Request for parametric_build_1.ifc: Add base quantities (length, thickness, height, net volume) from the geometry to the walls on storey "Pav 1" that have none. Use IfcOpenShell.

First a look at what the model holds.

```python
import ifcopenshell
import ifcopenshell.util.element
import ifcopenshell.util.unit

model = ifcopenshell.open("parametric_build_1.ifc")
print(model.schema)
for unit_type in ("LENGTHUNIT", "AREAUNIT", "VOLUMEUNIT"):
    print(unit_type, ifcopenshell.util.unit.calculate_unit_scale(model, unit_type))
storey = next(s for s in model.by_type("IfcBuildingStorey") if s.Name == "Pav 1")
walls = [e for e in ifcopenshell.util.element.get_decomposition(storey) if e.is_a("IfcWall")]
for e in sorted(walls, key=lambda e: e.id()):
    print(e.id(), e.is_a(), e.Name, list(ifcopenshell.util.element.get_psets(e, qtos_only=True)), sep=" | ")
```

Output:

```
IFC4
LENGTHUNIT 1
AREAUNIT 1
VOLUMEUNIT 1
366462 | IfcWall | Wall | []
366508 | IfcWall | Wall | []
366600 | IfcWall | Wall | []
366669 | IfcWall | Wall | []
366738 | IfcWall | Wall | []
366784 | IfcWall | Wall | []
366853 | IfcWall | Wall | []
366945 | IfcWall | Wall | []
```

```python
import ifcopenshell
import ifcopenshell.api.pset
import ifcopenshell.geom
import ifcopenshell.util.element
import ifcopenshell.util.shape
import ifcopenshell.util.unit

model = ifcopenshell.open("parametric_build_1.ifc")
unit_scale = ifcopenshell.util.unit.calculate_unit_scale(model)
volume_scale = ifcopenshell.util.unit.calculate_unit_scale(model, "VOLUMEUNIT")
settings = ifcopenshell.geom.settings()

storey = next(s for s in model.by_type("IfcBuildingStorey") if s.Name == "Pav 1")
walls = [e for e in ifcopenshell.util.element.get_decomposition(storey) if e.is_a("IfcWall")]

for e in sorted(walls, key=lambda e: e.id()):
    if ifcopenshell.util.element.get_psets(e, qtos_only=True, should_inherit=False):
        continue
    # Geometry comes back in metres, in the element's own axes.
    shape = ifcopenshell.geom.create_shape(settings, e)
    values = {
        "Length": ifcopenshell.util.shape.get_x(shape.geometry) / unit_scale,
        "Width": ifcopenshell.util.shape.get_y(shape.geometry) / unit_scale,
        "Height": ifcopenshell.util.shape.get_z(shape.geometry) / unit_scale,
        "NetVolume": ifcopenshell.util.shape.get_volume(shape.geometry) / volume_scale,
    }
    qto = ifcopenshell.api.pset.add_qto(model, product=e, name="Qto_WallBaseQuantities")
    ifcopenshell.api.pset.edit_qto(model, qto=qto, properties=values)
    print(e.id(), {k: round(v, 3) for k, v in values.items()})

model.write("parametric_build_1_rev.ifc")
```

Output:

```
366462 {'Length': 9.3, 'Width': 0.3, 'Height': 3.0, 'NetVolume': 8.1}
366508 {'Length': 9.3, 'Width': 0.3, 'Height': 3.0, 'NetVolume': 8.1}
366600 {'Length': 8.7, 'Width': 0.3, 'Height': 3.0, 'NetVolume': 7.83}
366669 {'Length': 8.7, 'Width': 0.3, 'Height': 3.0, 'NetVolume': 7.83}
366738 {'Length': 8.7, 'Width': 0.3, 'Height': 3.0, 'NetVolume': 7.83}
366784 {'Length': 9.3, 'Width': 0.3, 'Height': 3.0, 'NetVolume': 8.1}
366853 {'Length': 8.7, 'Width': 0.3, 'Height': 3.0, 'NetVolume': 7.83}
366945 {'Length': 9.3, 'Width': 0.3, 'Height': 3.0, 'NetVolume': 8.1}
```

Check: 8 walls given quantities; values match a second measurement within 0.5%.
